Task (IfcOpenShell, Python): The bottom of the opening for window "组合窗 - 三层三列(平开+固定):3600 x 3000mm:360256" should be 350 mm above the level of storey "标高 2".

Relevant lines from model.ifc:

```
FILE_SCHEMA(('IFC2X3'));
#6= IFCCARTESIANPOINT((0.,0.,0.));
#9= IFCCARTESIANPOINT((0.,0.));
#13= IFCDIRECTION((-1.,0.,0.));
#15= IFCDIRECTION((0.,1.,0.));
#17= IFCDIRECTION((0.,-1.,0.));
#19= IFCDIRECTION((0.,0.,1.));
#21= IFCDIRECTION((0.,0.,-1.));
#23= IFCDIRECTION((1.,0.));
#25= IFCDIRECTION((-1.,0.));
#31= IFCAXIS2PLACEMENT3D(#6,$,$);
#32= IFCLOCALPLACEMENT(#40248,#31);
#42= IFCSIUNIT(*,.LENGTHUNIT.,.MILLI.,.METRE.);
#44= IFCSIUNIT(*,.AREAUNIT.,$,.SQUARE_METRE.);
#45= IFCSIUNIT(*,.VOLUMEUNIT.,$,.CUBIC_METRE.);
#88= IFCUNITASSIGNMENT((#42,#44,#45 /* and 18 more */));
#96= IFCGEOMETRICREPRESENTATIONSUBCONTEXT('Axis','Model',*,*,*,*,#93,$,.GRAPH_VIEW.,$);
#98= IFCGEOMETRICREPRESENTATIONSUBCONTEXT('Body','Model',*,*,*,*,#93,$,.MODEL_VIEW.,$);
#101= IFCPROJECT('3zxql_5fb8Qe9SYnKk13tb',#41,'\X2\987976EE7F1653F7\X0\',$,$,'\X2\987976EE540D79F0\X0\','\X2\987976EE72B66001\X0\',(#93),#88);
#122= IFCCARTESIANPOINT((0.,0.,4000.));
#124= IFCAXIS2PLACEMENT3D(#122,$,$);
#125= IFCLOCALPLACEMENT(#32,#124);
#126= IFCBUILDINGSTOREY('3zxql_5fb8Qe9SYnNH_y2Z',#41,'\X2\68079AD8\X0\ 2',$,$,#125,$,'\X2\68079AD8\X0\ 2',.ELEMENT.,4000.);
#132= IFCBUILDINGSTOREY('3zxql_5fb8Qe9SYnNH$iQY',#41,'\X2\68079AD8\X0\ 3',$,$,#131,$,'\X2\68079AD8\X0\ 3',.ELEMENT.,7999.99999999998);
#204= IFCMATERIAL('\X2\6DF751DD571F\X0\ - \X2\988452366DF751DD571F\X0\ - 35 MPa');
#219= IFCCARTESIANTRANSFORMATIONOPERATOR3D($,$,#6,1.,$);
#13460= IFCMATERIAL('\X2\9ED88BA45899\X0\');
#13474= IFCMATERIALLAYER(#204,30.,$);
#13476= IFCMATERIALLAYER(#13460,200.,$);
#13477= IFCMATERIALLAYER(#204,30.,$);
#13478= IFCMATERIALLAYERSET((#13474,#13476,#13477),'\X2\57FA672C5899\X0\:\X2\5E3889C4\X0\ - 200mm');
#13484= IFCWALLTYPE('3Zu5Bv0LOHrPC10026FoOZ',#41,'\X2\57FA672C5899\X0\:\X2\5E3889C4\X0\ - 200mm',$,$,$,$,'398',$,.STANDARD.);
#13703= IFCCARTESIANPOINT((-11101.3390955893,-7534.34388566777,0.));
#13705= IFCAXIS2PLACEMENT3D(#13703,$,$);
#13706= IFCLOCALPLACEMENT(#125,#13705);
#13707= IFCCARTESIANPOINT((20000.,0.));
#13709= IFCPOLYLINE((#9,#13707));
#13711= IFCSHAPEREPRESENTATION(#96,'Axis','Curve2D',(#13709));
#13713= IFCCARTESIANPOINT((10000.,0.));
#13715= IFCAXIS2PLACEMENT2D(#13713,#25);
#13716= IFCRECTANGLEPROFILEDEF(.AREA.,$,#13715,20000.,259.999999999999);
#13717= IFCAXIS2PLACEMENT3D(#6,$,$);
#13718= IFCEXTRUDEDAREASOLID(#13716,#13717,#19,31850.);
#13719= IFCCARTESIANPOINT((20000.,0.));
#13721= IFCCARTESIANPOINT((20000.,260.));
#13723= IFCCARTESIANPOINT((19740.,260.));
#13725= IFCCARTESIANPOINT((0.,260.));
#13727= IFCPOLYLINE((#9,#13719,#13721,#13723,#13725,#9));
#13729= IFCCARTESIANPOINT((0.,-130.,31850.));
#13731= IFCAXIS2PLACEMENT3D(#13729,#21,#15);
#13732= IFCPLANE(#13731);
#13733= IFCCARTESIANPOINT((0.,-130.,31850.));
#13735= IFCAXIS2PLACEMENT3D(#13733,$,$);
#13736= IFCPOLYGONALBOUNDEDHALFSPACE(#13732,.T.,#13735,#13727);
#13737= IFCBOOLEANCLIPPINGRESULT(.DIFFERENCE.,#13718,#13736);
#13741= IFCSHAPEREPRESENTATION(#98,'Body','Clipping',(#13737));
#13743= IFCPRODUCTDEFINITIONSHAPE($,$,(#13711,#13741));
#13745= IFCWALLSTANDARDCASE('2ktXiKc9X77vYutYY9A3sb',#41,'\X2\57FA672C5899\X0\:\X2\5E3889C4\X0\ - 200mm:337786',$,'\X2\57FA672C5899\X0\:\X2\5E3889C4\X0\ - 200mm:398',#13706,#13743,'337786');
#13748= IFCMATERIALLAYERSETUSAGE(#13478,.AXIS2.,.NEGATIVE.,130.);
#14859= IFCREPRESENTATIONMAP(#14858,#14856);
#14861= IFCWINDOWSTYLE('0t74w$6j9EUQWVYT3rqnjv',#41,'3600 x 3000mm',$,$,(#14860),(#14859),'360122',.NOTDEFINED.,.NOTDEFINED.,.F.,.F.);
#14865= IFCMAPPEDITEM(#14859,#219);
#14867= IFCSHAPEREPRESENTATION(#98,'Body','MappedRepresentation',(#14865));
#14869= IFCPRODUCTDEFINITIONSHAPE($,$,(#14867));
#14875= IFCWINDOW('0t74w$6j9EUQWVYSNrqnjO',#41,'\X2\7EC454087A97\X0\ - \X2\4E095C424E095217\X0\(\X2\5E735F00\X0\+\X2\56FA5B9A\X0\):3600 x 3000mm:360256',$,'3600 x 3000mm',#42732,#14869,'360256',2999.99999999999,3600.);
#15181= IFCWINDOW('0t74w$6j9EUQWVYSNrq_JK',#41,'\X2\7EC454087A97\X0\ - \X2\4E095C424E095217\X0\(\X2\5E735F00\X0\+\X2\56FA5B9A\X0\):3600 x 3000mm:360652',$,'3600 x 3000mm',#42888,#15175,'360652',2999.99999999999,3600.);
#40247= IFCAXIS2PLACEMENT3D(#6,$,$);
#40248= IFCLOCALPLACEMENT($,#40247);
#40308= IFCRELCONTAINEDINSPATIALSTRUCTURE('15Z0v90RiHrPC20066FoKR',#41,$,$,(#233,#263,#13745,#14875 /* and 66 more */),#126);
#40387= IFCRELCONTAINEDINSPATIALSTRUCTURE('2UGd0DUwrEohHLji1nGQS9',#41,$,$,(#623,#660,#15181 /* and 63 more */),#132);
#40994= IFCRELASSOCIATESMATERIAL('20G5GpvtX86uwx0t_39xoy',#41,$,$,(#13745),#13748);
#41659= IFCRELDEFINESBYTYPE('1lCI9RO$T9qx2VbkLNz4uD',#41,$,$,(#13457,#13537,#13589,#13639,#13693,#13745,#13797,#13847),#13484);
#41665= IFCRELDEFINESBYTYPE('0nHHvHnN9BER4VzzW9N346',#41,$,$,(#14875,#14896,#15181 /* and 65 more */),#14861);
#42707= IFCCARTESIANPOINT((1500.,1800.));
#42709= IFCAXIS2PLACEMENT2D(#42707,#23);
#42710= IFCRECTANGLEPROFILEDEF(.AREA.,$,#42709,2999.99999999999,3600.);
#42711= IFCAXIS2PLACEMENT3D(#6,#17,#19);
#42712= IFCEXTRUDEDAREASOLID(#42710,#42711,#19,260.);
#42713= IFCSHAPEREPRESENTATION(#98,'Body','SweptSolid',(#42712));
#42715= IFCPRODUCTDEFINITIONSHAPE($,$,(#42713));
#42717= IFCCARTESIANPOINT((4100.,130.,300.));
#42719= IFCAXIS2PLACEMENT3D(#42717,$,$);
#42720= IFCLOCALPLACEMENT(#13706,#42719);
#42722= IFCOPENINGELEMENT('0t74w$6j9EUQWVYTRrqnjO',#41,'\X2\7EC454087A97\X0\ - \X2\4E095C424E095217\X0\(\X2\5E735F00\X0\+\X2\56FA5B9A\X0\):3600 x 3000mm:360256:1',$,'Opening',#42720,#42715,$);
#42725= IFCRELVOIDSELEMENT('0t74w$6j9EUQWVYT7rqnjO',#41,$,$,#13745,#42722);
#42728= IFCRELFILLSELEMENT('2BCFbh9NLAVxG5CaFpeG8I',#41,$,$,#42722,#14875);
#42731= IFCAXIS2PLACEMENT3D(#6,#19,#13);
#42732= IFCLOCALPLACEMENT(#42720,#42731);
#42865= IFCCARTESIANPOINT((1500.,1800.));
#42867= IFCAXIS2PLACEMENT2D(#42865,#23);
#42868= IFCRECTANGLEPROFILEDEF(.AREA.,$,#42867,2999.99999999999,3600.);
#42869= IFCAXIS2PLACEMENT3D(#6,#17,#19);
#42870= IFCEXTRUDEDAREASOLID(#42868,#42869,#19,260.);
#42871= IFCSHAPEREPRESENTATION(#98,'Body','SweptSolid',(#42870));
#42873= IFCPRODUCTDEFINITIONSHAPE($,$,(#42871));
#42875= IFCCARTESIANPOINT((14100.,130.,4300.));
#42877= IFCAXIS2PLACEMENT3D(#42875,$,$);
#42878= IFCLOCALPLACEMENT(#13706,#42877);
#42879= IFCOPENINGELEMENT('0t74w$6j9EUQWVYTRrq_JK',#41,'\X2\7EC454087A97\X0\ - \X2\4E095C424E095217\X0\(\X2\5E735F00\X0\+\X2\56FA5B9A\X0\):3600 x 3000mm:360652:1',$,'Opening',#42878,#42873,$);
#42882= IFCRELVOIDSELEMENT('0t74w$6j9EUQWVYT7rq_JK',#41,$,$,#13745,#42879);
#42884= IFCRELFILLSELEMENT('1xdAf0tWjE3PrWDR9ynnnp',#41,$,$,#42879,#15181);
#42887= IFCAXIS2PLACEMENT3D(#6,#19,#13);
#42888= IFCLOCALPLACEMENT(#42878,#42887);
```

```python
import numpy as np
import ifcopenshell
import ifcopenshell.api.geometry
import ifcopenshell.geom
import ifcopenshell.util.element
import ifcopenshell.util.placement
import ifcopenshell.util.shape
import ifcopenshell.util.unit

model = ifcopenshell.open("model.ifc")
unit_scale = ifcopenshell.util.unit.calculate_unit_scale(model)

window = model.by_guid("0t74w$6j9EUQWVYSNrqnjO")
opening = window.FillsVoids[0].RelatingOpeningElement
storey = ifcopenshell.util.element.get_container(window, ifc_class="IfcBuildingStorey")
level = ifcopenshell.util.placement.get_local_placement(storey.ObjectPlacement)[2, 3]

# The opening's origin need not be at the sill, so measure its lowest point.
shape = ifcopenshell.geom.create_shape(ifcopenshell.geom.settings(), opening)
bottom = ifcopenshell.util.shape.get_shape_bottom_elevation(shape, shape.geometry) / unit_scale
dz = level + 350.0 - bottom

shift = np.array([0.0, 0.0, dz])
# The window is placed relative to its opening, so it follows when the opening moves.
matrix = ifcopenshell.util.placement.get_local_placement(opening.ObjectPlacement)
matrix[:3, 3] += shift
ifcopenshell.api.geometry.edit_object_placement(
    model, product=opening, matrix=matrix, is_si=False, should_transform_children=True
)

print(f"moved by {dz * unit_scale:+.3f} m")

model.write("model-out.ifc")
```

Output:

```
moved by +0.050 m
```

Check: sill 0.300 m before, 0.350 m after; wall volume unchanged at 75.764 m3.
